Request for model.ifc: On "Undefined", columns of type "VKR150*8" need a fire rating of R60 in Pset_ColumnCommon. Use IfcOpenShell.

First a look at what the model holds.

```python
import ifcopenshell
import ifcopenshell.util.element

model = ifcopenshell.open("model.ifc")
print(model.schema)
storey = next(s for s in model.by_type("IfcBuildingStorey") if s.Name == "Undefined")
columns = [e for e in ifcopenshell.util.element.get_decomposition(storey) if e.is_a("IfcColumn")]
seen = {}
for e in columns:
    element_type = ifcopenshell.util.element.get_type(e)
    key = (element_type.Name if element_type != e and element_type else None, ifcopenshell.util.element.get_pset(e, "Pset_ColumnCommon", "FireRating"))
    seen[key] = seen.get(key, 0) + 1
for (name, value), count in sorted(seen.items(), key=str):
    print(count, "x", name, "|", value)
```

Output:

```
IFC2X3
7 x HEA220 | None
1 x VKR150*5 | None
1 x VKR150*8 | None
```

```python
import ifcopenshell
import ifcopenshell.api.pset
import ifcopenshell.util.element

model = ifcopenshell.open("model.ifc")

storey = next(s for s in model.by_type("IfcBuildingStorey") if s.Name == "Undefined")
columns = [e for e in ifcopenshell.util.element.get_decomposition(storey) if e.is_a("IfcColumn")]

count = 0
for e in columns:
    element_type = ifcopenshell.util.element.get_type(e)
    if element_type in (None, e) or element_type.Name != "VKR150*8":
        continue
    found = ifcopenshell.util.element.get_pset(e, "Pset_ColumnCommon", should_inherit=False)
    if found:
        pset = model.by_id(found["id"])
        if len(ifcopenshell.util.element.get_elements_by_pset(pset)) > 1:
            pset = ifcopenshell.api.pset.unshare_pset(model, products=[e], pset=pset)[0]
    else:
        pset = ifcopenshell.api.pset.add_pset(model, product=e, name="Pset_ColumnCommon")
    ifcopenshell.api.pset.edit_pset(model, pset=pset, properties={"FireRating": "R60"})
    count += 1

print(count, "columns updated")

model.write("model-out.ifc")
```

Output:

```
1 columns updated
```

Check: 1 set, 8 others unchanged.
